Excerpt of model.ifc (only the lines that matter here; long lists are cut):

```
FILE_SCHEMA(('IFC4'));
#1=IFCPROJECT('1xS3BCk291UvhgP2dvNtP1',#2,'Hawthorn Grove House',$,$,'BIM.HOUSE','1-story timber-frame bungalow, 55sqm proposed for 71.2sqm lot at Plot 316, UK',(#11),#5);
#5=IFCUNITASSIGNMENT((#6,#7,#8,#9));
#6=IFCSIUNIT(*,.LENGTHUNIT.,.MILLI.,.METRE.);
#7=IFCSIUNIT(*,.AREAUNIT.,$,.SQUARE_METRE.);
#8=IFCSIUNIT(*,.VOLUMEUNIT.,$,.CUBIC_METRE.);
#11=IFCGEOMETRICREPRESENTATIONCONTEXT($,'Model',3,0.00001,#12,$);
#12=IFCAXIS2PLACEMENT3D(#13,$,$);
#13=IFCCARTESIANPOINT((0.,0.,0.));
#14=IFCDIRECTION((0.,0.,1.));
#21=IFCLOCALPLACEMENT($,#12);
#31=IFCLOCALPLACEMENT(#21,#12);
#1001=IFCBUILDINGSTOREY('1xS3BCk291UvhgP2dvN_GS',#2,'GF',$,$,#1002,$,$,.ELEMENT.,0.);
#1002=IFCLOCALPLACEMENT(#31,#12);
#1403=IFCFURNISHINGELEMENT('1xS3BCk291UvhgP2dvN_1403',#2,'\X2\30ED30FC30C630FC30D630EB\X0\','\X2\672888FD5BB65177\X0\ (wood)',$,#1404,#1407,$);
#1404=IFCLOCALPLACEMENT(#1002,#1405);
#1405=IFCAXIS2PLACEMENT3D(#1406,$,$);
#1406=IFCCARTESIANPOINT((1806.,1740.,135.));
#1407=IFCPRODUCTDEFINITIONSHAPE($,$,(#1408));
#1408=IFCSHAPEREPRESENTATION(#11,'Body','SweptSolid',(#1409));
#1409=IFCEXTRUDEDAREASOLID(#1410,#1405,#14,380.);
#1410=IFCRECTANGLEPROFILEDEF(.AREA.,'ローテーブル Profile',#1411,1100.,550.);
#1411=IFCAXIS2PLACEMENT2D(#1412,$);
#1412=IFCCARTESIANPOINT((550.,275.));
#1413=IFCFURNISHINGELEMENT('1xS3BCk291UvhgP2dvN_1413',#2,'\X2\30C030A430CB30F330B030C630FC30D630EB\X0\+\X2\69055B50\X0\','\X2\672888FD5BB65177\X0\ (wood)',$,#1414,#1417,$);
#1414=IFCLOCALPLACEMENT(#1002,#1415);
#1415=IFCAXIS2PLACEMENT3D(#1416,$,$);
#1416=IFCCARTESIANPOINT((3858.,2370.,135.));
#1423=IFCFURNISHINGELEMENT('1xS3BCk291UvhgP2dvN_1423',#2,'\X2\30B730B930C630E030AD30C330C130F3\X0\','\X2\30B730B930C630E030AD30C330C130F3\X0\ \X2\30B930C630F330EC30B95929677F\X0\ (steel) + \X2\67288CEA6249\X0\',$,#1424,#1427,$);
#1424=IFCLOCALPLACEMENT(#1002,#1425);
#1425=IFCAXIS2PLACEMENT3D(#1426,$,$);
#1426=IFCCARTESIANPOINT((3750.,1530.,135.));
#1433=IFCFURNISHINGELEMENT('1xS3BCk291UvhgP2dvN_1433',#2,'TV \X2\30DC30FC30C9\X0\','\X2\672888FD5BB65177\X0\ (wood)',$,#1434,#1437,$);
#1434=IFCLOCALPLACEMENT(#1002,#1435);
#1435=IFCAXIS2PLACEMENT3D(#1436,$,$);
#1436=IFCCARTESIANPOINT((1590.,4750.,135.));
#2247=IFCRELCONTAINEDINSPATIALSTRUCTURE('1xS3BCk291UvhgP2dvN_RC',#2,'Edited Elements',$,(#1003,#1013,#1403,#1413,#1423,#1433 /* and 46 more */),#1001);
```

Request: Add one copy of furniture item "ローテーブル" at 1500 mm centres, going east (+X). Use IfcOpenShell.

```python
import numpy as np
import ifcopenshell
import ifcopenshell.api.geometry
import ifcopenshell.api.root
import ifcopenshell.util.element
import ifcopenshell.util.placement
import ifcopenshell.util.unit

model = ifcopenshell.open("model.ifc")
unit_scale = ifcopenshell.util.unit.calculate_unit_scale(model)


def reuse_history(source, copy):
    """copy_class also copies each property set's owner history, people and application; keep the originals."""
    for rel in copy.IsDefinedBy:
        if rel.is_a("IfcRelDefinesByProperties") and (history := rel.RelatingPropertyDefinition.OwnerHistory):
            rel.RelatingPropertyDefinition.OwnerHistory = source.OwnerHistory
            ifcopenshell.util.element.remove_deep2(model, history)


source = model.by_id(1403)
base = ifcopenshell.util.placement.get_local_placement(source.ObjectPlacement)
step = np.array([1.0, 0.0, 0.0]) * 1.5 / unit_scale

for i in range(1, 2):
    copy = ifcopenshell.api.root.copy_class(model, product=source)
    copy.Representation = ifcopenshell.util.element.copy_deep(
        model, source.Representation, exclude=["IfcGeometricRepresentationContext", "IfcRepresentationMap"]
    )
    reuse_history(source, copy)
    matrix = base.copy()
    matrix[:3, 3] += i * step
    print("added at", matrix[:3, 3].round(3) + 0.0)
    ifcopenshell.api.geometry.edit_object_placement(model, product=copy, matrix=matrix, is_si=False)

model.write("model_v2.ifc")
```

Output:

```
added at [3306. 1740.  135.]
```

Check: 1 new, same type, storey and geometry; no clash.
